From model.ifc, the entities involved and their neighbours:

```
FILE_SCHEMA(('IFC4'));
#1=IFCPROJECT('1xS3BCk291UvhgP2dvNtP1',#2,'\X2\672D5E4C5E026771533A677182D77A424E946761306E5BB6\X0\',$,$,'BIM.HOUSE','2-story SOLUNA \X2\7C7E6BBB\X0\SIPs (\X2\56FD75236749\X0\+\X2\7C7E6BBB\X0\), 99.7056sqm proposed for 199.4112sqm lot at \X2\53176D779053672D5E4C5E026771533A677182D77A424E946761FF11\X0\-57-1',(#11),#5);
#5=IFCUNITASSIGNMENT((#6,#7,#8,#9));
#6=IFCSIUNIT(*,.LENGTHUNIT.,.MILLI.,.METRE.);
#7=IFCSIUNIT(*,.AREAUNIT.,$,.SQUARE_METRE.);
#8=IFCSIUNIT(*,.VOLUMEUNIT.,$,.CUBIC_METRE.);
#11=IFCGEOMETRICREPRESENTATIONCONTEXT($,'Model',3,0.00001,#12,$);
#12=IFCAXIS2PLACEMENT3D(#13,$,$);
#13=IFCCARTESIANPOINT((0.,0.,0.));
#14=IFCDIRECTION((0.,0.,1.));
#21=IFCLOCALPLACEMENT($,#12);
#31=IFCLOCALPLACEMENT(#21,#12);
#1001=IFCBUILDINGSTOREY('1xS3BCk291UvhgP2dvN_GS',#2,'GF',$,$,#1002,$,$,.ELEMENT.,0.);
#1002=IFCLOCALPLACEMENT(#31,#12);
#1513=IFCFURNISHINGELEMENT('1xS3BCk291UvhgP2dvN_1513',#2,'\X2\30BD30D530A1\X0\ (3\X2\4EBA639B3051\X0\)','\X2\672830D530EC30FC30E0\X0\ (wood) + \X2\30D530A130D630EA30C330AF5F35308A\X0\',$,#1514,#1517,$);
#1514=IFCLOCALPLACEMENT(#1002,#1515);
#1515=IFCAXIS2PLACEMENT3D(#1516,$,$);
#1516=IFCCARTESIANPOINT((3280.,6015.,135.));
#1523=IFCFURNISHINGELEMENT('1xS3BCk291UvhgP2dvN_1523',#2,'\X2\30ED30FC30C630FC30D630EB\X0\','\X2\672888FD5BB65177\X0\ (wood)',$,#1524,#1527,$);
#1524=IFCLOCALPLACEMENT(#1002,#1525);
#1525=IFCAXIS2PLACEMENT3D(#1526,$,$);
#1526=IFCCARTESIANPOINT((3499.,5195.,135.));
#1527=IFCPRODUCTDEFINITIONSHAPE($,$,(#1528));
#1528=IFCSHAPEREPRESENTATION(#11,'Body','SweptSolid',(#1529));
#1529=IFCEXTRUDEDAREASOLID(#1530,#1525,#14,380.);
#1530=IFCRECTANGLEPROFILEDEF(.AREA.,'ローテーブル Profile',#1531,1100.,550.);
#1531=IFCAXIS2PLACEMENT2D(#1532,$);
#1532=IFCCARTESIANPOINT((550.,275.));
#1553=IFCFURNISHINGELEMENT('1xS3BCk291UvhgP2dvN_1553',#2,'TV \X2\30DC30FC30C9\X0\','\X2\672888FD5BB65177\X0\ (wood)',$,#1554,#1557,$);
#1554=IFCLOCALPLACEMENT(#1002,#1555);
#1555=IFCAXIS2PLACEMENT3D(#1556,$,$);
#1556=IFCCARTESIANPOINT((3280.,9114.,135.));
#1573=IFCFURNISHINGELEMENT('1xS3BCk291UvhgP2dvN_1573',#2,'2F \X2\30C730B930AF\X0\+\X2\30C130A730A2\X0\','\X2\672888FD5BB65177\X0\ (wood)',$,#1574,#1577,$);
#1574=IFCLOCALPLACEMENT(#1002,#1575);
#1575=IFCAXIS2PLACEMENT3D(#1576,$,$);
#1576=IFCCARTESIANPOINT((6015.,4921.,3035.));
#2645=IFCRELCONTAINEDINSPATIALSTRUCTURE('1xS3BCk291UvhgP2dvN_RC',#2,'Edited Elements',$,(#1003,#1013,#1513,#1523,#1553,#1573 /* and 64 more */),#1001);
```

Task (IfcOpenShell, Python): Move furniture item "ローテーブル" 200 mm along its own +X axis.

```python
import ifcopenshell
import ifcopenshell.api.geometry
import ifcopenshell.util.placement

model = ifcopenshell.open("model.ifc")

item = model.by_id(1523)
matrix = ifcopenshell.util.placement.get_local_placement(item.ObjectPlacement)
matrix[:3, 3] += matrix[:3, 0] * 200.0
ifcopenshell.api.geometry.edit_object_placement(model, product=item, matrix=matrix, is_si=False)

print(ifcopenshell.util.placement.get_local_placement(item.ObjectPlacement).round(3) + 0.0)

model.write("model_rev.ifc")
```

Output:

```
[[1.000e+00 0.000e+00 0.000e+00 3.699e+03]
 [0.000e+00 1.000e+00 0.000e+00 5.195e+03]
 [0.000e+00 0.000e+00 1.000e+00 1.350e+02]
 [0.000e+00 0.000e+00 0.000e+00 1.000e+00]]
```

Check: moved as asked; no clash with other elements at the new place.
